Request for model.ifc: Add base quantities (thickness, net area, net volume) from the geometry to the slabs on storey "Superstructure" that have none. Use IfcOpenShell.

First a look at what the model holds.

```python
import ifcopenshell
import ifcopenshell.util.element
import ifcopenshell.util.unit

model = ifcopenshell.open("model.ifc")
print(model.schema)
for unit_type in ("LENGTHUNIT", "AREAUNIT", "VOLUMEUNIT"):
    print(unit_type, ifcopenshell.util.unit.calculate_unit_scale(model, unit_type))
storey = next(s for s in model.by_type("IfcBuildingStorey") if s.Name == "Superstructure")
slabs = [e for e in ifcopenshell.util.element.get_decomposition(storey) if e.is_a("IfcSlab")]
for e in sorted(slabs, key=lambda e: e.id()):
    print(e.id(), e.is_a(), e.Name, list(ifcopenshell.util.element.get_psets(e, qtos_only=True)), sep=" | ")
```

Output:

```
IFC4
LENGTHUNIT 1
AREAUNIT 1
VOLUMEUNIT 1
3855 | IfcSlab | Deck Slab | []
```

```python
import ifcopenshell
import ifcopenshell.api.pset
import ifcopenshell.geom
import ifcopenshell.util.element
import ifcopenshell.util.shape
import ifcopenshell.util.unit

model = ifcopenshell.open("model.ifc")
unit_scale = ifcopenshell.util.unit.calculate_unit_scale(model)
area_scale = ifcopenshell.util.unit.calculate_unit_scale(model, "AREAUNIT")
volume_scale = ifcopenshell.util.unit.calculate_unit_scale(model, "VOLUMEUNIT")
settings = ifcopenshell.geom.settings()

storey = next(s for s in model.by_type("IfcBuildingStorey") if s.Name == "Superstructure")
slabs = [e for e in ifcopenshell.util.element.get_decomposition(storey) if e.is_a("IfcSlab")]

for e in sorted(slabs, key=lambda e: e.id()):
    if ifcopenshell.util.element.get_psets(e, qtos_only=True, should_inherit=False):
        continue
    # Geometry comes back in metres, in the element's own axes.
    shape = ifcopenshell.geom.create_shape(settings, e)
    values = {
        "Width": ifcopenshell.util.shape.get_z(shape.geometry) / unit_scale,
        "NetArea": ifcopenshell.util.shape.get_footprint_area(shape.geometry) / area_scale,
        "NetVolume": ifcopenshell.util.shape.get_volume(shape.geometry) / volume_scale,
    }
    qto = ifcopenshell.api.pset.add_qto(model, product=e, name="Qto_SlabBaseQuantities")
    ifcopenshell.api.pset.edit_qto(model, qto=qto, properties=values)
    print(e.id(), {k: round(v, 3) for k, v in values.items()})

model.write("model_rev.ifc")
```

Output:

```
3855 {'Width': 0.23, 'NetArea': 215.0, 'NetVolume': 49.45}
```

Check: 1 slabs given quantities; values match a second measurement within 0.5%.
